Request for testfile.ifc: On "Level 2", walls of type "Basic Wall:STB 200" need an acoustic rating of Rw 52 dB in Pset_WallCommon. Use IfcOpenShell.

First a look at what the model holds.

```python
import ifcopenshell
import ifcopenshell.util.element

model = ifcopenshell.open("testfile.ifc")
print(model.schema)
storey = next(s for s in model.by_type("IfcBuildingStorey") if s.Name == "Level 2")
walls = [e for e in ifcopenshell.util.element.get_decomposition(storey) if e.is_a("IfcWall")]
seen = {}
for e in walls:
    element_type = ifcopenshell.util.element.get_type(e)
    key = (element_type.Name if element_type != e and element_type else None, ifcopenshell.util.element.get_pset(e, "Pset_WallCommon", "AcousticRating"))
    seen[key] = seen.get(key, 0) + 1
for (name, value), count in sorted(seen.items(), key=str):
    print(count, "x", name, "|", value)
```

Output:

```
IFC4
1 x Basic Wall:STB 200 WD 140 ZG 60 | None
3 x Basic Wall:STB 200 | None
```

```python
import ifcopenshell
import ifcopenshell.api.pset
import ifcopenshell.util.element

model = ifcopenshell.open("testfile.ifc")

storey = next(s for s in model.by_type("IfcBuildingStorey") if s.Name == "Level 2")
walls = [e for e in ifcopenshell.util.element.get_decomposition(storey) if e.is_a("IfcWall")]

count = 0
for e in walls:
    element_type = ifcopenshell.util.element.get_type(e)
    if element_type in (None, e) or element_type.Name != "Basic Wall:STB 200":
        continue
    # add_pset returns the element's existing set when there is one.
    pset = ifcopenshell.api.pset.add_pset(model, product=e, name="Pset_WallCommon")
    ifcopenshell.api.pset.edit_pset(model, pset=pset, properties={"AcousticRating": "Rw 52 dB"})
    count += 1

print(count, "walls updated")

model.write("testfile_updated.ifc")
```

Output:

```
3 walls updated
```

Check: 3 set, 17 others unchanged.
